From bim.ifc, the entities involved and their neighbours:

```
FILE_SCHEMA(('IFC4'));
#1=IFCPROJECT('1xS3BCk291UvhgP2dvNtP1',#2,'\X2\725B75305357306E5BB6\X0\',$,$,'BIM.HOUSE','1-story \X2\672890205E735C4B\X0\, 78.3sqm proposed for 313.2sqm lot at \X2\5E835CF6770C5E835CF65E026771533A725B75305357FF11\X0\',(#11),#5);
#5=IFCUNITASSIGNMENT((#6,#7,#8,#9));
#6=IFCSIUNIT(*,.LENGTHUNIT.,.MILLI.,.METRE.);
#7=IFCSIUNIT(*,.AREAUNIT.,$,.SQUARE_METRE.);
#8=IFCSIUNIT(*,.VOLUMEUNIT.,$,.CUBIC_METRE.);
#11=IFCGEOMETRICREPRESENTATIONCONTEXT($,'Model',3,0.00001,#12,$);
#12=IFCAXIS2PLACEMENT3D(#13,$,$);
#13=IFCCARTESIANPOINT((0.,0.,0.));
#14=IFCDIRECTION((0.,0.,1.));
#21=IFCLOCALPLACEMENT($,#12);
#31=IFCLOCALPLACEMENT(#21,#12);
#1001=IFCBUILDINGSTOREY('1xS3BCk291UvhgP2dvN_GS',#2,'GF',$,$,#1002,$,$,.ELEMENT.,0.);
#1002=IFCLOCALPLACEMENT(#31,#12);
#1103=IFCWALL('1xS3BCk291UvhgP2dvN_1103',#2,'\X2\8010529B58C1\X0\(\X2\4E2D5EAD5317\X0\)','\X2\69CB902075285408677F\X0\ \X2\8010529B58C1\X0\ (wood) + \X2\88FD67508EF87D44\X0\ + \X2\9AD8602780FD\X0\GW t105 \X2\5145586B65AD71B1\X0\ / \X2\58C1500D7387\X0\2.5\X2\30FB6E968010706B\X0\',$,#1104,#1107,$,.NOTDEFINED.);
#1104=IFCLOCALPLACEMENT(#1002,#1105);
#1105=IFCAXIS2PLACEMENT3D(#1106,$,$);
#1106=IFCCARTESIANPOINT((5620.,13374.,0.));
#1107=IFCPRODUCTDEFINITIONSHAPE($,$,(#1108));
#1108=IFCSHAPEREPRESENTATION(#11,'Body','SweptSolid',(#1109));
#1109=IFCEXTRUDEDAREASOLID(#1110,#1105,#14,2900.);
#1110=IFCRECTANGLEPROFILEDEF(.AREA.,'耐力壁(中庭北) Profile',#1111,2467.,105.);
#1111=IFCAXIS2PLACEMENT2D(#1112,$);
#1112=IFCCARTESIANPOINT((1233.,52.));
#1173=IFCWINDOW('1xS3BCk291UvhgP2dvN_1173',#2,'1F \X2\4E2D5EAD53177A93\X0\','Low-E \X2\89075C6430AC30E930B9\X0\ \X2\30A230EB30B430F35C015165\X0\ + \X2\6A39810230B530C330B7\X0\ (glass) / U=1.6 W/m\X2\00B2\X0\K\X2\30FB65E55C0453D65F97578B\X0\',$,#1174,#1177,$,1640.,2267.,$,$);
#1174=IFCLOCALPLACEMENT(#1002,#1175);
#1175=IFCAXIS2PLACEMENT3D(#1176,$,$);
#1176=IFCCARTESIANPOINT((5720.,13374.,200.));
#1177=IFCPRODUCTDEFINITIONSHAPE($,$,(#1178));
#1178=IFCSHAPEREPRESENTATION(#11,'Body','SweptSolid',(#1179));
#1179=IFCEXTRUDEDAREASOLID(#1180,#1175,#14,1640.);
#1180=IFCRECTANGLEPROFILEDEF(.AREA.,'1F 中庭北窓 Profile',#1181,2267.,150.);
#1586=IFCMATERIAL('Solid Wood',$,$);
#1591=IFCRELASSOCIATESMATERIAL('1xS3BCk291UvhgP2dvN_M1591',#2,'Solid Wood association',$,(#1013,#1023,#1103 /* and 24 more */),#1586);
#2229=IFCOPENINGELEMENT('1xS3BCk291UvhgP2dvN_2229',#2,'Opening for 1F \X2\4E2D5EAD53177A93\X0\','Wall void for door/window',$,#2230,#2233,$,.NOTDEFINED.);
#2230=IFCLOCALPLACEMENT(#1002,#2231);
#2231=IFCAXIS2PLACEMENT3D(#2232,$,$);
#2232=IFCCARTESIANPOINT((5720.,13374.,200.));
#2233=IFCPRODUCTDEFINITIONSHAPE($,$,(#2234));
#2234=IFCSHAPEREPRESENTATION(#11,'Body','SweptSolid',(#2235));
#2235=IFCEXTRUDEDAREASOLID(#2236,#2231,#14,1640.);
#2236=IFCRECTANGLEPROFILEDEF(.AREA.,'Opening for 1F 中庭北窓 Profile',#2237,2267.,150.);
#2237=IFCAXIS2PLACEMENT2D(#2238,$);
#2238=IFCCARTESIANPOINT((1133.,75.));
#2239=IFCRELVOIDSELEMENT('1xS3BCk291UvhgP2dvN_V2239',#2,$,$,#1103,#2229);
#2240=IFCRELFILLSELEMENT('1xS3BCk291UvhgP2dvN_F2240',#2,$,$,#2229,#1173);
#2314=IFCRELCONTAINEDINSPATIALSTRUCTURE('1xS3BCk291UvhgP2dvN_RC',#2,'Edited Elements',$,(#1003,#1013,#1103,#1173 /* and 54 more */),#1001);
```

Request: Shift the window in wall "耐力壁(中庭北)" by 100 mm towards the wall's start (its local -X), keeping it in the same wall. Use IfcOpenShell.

```python
import ifcopenshell
import ifcopenshell.api.geometry
import ifcopenshell.util.placement
import ifcopenshell.util.unit

model = ifcopenshell.open("bim.ifc")
unit_scale = ifcopenshell.util.unit.calculate_unit_scale(model)

window = model.by_id(1173)
opening = window.FillsVoids[0].RelatingOpeningElement
wall = opening.VoidsElements[0].RelatingBuildingElement

wall_matrix = ifcopenshell.util.placement.get_local_placement(wall.ObjectPlacement)
shift = wall_matrix[:3, 0] * -0.1 / unit_scale
before = ifcopenshell.util.placement.get_local_placement(window.ObjectPlacement)[:3, 3].copy()

# The window is not placed relative to its opening, so move both.
for product in (opening, window):
    matrix = ifcopenshell.util.placement.get_local_placement(product.ObjectPlacement)
    matrix[:3, 3] += shift
    ifcopenshell.api.geometry.edit_object_placement(model, product=product, matrix=matrix, is_si=False)

after = ifcopenshell.util.placement.get_local_placement(window.ObjectPlacement)[:3, 3]
print("window moved by", (after - before).round(3) + 0.0)

model.write("bim-out.ifc")
```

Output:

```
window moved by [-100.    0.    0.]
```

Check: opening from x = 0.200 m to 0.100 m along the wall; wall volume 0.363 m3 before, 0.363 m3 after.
